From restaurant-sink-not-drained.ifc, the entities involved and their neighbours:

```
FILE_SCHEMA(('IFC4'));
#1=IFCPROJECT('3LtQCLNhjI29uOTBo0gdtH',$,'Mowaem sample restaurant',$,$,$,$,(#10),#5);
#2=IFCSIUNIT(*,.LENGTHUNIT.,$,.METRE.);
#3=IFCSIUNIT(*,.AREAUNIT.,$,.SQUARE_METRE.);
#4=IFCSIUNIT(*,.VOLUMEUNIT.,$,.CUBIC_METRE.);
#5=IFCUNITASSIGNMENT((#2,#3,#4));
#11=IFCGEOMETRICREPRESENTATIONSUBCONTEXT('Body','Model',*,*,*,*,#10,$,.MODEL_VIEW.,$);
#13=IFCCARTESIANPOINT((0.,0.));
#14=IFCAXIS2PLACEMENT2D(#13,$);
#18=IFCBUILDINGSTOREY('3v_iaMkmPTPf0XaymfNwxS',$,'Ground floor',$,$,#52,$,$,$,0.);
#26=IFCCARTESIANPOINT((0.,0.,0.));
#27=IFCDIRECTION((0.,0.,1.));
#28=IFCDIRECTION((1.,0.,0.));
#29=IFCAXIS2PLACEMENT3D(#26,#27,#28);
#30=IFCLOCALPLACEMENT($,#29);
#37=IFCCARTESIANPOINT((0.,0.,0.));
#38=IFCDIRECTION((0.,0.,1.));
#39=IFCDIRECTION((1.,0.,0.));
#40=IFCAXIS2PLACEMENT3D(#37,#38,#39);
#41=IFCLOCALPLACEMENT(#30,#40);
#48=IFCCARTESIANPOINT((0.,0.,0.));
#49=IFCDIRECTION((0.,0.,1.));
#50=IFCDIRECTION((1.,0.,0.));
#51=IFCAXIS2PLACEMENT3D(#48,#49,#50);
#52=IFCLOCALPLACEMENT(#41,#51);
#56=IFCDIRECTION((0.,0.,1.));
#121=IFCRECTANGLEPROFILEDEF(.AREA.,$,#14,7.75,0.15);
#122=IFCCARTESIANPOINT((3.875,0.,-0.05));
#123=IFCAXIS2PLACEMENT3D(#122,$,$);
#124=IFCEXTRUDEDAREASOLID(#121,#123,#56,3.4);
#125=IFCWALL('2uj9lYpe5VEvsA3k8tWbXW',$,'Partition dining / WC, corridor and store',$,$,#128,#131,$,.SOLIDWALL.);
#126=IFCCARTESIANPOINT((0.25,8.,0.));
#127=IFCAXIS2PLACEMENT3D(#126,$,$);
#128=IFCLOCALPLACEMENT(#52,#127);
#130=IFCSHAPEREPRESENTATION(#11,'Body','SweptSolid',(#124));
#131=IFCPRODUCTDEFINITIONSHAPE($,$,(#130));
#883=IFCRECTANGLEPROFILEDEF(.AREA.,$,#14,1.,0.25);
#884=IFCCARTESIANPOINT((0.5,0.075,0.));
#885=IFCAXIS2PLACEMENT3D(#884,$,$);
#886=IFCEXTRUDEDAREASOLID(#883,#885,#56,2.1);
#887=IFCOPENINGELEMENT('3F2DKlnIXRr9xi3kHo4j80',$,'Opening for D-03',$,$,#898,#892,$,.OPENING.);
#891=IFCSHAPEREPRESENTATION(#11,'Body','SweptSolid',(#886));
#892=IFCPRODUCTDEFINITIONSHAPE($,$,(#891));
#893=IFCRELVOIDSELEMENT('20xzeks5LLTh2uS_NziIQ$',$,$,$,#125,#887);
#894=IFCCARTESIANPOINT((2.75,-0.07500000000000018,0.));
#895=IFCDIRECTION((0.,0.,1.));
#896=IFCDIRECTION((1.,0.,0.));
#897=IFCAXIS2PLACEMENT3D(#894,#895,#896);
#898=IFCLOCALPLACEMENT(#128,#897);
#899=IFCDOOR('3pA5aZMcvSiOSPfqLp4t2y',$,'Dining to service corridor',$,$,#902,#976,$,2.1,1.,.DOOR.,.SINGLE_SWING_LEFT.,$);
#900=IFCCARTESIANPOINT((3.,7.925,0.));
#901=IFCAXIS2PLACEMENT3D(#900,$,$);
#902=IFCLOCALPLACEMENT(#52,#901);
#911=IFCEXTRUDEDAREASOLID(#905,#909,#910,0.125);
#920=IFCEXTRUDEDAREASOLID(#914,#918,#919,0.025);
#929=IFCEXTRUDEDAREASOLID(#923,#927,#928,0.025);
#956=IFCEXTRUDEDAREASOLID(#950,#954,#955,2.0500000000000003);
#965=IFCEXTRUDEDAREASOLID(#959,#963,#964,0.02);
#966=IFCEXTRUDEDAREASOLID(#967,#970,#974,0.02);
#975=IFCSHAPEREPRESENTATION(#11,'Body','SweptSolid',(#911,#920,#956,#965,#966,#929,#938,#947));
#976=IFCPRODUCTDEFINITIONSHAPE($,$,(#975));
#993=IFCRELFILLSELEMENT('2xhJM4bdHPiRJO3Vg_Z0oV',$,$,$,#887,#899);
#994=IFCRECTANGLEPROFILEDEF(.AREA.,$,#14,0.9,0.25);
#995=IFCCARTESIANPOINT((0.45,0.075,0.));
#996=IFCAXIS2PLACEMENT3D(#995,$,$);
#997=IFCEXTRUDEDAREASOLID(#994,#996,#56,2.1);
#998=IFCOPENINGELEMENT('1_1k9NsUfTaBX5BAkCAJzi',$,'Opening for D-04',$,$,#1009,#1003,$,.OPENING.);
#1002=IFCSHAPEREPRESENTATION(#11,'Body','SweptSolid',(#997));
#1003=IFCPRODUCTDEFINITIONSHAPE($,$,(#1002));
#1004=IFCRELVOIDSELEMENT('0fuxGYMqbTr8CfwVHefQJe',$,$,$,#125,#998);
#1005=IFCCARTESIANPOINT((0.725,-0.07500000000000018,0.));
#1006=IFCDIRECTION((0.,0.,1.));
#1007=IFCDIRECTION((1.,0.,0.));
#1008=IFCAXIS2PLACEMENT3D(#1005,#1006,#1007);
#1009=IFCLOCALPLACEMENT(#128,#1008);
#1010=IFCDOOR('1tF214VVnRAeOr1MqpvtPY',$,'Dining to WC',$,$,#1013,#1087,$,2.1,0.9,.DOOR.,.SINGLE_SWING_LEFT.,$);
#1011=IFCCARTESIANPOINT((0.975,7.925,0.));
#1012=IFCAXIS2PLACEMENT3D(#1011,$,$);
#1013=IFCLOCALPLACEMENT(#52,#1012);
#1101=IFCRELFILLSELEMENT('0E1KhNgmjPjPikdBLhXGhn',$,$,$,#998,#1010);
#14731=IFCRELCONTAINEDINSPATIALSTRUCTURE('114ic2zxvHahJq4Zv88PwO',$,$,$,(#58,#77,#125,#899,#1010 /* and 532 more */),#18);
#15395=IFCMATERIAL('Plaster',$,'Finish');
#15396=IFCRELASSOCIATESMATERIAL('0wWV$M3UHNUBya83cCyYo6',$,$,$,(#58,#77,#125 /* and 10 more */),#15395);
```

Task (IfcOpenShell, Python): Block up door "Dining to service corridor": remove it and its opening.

```python
import ifcopenshell
import ifcopenshell.api.feature
import ifcopenshell.api.root
import ifcopenshell.geom
import ifcopenshell.util.shape

model = ifcopenshell.open("restaurant-sink-not-drained.ifc")
settings = ifcopenshell.geom.settings()


def volume(element):
    """Net volume in cubic metres, openings subtracted."""
    shape = ifcopenshell.geom.create_shape(settings, element)
    return ifcopenshell.util.shape.get_volume(shape.geometry)


door = model.by_guid("3pA5aZMcvSiOSPfqLp4t2y")
opening = door.FillsVoids[0].RelatingOpeningElement
wall = opening.VoidsElements[0].RelatingBuildingElement
before = volume(wall)

ifcopenshell.api.root.remove_product(model, product=door)
ifcopenshell.api.feature.remove_feature(model, feature=opening)

after = volume(wall)

print(f"wall volume {before:.3f} -> {after:.3f} m3")

model.write("restaurant-sink-not-drained_edited.ifc")
```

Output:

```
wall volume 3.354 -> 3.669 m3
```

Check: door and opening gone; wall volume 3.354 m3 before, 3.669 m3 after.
